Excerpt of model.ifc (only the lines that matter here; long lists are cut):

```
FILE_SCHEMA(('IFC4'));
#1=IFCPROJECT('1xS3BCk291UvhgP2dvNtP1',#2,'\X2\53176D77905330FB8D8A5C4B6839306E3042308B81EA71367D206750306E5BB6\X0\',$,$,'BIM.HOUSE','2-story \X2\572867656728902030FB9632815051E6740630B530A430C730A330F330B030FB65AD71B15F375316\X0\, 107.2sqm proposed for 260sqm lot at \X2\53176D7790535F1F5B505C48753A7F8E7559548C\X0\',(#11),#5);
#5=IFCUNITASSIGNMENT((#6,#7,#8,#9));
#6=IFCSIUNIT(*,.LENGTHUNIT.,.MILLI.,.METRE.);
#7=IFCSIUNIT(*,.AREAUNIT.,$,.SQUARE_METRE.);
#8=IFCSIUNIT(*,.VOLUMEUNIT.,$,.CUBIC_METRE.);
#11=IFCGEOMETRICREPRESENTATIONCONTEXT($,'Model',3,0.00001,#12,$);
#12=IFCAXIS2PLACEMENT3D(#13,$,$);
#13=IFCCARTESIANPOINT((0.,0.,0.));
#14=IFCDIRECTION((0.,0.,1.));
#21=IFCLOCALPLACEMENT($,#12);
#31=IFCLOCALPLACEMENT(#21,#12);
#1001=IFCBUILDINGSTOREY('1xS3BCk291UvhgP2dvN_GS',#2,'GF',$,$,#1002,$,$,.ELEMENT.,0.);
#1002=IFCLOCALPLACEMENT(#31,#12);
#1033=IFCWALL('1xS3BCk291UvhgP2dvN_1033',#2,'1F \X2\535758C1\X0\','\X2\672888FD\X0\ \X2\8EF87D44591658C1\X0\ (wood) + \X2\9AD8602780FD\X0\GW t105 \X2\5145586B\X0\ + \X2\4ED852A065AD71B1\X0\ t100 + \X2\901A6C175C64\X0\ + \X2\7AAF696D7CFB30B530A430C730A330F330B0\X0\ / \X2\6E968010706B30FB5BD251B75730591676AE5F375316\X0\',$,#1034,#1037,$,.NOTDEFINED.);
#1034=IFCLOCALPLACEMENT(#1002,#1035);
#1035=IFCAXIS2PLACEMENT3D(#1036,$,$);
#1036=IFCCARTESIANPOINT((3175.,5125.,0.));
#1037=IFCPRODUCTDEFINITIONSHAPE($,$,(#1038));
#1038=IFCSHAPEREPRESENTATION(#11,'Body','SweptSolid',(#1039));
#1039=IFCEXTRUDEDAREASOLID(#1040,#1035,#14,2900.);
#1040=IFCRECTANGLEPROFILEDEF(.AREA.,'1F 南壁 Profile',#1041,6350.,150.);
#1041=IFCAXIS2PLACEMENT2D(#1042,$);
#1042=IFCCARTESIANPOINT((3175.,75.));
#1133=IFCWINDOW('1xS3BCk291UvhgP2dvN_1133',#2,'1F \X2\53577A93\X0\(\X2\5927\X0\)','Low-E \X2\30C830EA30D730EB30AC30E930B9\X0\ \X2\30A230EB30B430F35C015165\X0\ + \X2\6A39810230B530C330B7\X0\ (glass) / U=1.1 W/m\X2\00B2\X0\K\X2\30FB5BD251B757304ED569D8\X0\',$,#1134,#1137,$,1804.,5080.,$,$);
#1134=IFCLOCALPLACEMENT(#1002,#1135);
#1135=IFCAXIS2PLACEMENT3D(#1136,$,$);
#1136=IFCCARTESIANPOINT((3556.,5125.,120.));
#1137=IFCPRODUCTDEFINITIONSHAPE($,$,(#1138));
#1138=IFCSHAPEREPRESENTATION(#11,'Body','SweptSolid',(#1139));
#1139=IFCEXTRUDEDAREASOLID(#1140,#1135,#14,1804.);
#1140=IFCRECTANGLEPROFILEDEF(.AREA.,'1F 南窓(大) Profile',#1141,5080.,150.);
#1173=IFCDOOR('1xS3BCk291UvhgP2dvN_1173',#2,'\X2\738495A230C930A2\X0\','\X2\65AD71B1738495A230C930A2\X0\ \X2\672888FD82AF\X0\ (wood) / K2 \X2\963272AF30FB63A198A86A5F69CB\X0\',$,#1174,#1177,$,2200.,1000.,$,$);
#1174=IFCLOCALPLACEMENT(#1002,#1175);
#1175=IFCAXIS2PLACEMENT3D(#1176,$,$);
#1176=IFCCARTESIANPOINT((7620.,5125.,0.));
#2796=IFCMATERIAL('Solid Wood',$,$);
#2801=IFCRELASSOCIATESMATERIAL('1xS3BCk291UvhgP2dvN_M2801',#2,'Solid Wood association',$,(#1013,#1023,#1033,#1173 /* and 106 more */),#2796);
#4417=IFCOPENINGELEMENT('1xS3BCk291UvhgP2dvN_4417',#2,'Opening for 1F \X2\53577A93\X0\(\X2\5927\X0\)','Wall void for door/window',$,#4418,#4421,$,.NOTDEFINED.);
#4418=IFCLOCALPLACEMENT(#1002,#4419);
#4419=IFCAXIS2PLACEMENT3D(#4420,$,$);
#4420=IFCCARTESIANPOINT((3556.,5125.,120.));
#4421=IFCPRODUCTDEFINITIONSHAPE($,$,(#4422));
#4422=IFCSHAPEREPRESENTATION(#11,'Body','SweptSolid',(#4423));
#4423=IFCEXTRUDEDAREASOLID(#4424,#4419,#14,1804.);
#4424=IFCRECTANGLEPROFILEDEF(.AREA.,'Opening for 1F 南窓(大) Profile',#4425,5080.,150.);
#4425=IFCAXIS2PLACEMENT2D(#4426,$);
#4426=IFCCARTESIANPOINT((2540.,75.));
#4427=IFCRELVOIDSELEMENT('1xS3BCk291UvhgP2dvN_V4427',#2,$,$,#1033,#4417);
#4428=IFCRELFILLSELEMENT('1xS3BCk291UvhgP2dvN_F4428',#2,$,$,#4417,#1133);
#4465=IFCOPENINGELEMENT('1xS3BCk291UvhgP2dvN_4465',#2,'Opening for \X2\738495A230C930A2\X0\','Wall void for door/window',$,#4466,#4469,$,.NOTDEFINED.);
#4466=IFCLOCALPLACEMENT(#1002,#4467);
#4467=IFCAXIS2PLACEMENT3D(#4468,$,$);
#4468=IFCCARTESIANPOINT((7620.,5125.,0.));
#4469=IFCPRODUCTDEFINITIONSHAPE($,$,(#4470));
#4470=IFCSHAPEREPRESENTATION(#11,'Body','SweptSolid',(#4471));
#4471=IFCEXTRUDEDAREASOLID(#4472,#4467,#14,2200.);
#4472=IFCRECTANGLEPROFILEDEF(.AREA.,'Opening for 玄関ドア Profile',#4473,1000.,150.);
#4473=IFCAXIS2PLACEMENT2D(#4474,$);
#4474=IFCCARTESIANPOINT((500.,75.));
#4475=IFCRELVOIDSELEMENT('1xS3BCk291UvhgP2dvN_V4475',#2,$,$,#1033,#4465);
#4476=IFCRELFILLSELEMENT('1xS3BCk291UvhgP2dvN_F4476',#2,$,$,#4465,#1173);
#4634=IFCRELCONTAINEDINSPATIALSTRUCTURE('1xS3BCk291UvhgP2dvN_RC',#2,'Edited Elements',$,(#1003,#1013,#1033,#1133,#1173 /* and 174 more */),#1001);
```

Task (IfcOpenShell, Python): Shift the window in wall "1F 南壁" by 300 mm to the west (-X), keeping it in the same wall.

```python
import ifcopenshell
import ifcopenshell.api.geometry
import ifcopenshell.util.placement
import ifcopenshell.util.unit

model = ifcopenshell.open("model.ifc")
unit_scale = ifcopenshell.util.unit.calculate_unit_scale(model)

window = model.by_id(1133)
opening = window.FillsVoids[0].RelatingOpeningElement
wall = opening.VoidsElements[0].RelatingBuildingElement

wall_matrix = ifcopenshell.util.placement.get_local_placement(wall.ObjectPlacement)
shift = wall_matrix[:3, 0] * -0.3 / unit_scale
before = ifcopenshell.util.placement.get_local_placement(window.ObjectPlacement)[:3, 3].copy()

# The window is not placed relative to its opening, so move both.
for product in (opening, window):
    matrix = ifcopenshell.util.placement.get_local_placement(product.ObjectPlacement)
    matrix[:3, 3] += shift
    ifcopenshell.api.geometry.edit_object_placement(model, product=product, matrix=matrix, is_si=False)

after = ifcopenshell.util.placement.get_local_placement(window.ObjectPlacement)[:3, 3]
print("window moved by", (after - before).round(3) + 0.0)

model.write("model_v2.ifc")
```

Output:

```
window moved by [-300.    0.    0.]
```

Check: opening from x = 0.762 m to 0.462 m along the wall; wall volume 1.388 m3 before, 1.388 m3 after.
